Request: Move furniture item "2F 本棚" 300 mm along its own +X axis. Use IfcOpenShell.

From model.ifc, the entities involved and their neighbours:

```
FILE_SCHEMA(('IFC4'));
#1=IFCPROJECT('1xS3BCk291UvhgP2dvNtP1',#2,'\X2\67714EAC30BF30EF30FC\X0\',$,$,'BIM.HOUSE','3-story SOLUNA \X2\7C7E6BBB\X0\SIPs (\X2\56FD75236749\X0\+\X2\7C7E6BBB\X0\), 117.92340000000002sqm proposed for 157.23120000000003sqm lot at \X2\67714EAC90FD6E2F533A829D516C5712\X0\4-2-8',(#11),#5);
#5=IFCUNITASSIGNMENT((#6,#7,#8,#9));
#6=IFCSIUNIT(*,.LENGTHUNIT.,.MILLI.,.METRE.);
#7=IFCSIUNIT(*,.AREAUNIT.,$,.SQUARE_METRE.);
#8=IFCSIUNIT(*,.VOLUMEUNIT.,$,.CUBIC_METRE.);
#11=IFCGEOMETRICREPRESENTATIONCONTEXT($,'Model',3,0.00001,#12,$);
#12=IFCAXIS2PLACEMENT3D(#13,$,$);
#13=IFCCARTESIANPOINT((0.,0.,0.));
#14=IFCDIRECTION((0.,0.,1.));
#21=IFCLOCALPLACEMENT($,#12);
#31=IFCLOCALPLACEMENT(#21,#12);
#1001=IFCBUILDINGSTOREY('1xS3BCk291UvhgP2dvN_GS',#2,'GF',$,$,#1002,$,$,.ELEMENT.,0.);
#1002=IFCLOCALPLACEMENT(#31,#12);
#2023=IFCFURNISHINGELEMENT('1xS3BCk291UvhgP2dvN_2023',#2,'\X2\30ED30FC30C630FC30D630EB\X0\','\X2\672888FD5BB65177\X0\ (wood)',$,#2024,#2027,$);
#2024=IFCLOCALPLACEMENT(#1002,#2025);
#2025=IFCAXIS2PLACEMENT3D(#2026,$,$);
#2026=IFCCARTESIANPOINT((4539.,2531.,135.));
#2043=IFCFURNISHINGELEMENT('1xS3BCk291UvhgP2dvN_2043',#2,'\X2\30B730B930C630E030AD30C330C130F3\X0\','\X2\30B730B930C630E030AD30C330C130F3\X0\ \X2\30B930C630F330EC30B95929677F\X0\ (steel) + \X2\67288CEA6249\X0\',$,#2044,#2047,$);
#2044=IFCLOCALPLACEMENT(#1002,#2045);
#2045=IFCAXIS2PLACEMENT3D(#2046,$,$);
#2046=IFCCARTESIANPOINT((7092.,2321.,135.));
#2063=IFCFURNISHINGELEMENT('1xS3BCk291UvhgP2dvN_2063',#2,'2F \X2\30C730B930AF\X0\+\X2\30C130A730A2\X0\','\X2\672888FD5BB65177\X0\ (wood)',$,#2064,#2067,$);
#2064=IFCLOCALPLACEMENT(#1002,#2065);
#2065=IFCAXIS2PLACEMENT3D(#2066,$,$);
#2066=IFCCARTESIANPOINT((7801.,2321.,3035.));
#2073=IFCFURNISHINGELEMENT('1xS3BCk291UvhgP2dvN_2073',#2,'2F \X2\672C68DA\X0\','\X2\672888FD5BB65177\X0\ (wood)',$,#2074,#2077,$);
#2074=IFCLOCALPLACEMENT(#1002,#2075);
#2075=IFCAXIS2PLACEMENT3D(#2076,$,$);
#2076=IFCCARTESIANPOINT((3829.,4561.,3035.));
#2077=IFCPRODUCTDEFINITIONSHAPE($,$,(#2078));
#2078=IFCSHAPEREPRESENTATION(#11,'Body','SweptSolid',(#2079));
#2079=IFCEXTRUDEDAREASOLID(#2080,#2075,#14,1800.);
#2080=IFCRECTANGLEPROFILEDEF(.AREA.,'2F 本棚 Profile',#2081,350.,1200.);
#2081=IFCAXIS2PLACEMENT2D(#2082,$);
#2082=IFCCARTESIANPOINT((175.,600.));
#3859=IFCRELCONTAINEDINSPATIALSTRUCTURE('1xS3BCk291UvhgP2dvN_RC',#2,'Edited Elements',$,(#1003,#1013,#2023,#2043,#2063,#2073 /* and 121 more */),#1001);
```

```python
import ifcopenshell
import ifcopenshell.api.geometry
import ifcopenshell.util.placement

model = ifcopenshell.open("model.ifc")

item = model.by_guid("1xS3BCk291UvhgP2dvN_2073")
matrix = ifcopenshell.util.placement.get_local_placement(item.ObjectPlacement)
matrix[:3, 3] += matrix[:3, 0] * 300.0
ifcopenshell.api.geometry.edit_object_placement(model, product=item, matrix=matrix, is_si=False)

print(ifcopenshell.util.placement.get_local_placement(item.ObjectPlacement).round(3) + 0.0)

model.write("model_edited.ifc")
```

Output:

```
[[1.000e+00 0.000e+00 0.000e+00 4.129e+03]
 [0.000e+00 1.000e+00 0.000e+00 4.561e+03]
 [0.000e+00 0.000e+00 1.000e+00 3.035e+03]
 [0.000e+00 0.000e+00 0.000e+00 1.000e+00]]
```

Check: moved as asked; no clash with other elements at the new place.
